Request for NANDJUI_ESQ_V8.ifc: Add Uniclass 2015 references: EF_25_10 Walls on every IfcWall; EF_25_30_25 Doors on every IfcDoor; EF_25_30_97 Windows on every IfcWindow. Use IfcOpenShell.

First a look at what the model holds.

```python
import ifcopenshell

model = ifcopenshell.open("NANDJUI_ESQ_V8.ifc")
print(model.schema)
print("classifications:", [c.Name for c in model.by_type("IfcClassification")])
for ifc_class in ("IfcDoor", "IfcRoof", "IfcStair", "IfcWall", "IfcWindow"):
    print(ifc_class, len(model.by_type(ifc_class)))
```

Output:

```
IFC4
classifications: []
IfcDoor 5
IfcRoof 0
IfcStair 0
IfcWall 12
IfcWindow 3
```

```python
import ifcopenshell
import ifcopenshell.api.classification

model = ifcopenshell.open("NANDJUI_ESQ_V8.ifc")

system = ifcopenshell.api.classification.add_classification(model, classification="Uniclass 2015")

codes = {
    "IfcWall": ("EF_25_10", "Walls"),
    "IfcDoor": ("EF_25_30_25", "Doors"),
    "IfcWindow": ("EF_25_30_97", "Windows"),
}
for ifc_class, (code, name) in codes.items():
    products = model.by_type(ifc_class)
    ifcopenshell.api.classification.add_reference(
        model, products=products, classification=system, identification=code, name=name
    )
    print(code, len(products))

model.write("NANDJUI_ESQ_V8_updated.ifc")
```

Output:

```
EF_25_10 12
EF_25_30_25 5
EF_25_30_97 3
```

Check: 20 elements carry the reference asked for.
